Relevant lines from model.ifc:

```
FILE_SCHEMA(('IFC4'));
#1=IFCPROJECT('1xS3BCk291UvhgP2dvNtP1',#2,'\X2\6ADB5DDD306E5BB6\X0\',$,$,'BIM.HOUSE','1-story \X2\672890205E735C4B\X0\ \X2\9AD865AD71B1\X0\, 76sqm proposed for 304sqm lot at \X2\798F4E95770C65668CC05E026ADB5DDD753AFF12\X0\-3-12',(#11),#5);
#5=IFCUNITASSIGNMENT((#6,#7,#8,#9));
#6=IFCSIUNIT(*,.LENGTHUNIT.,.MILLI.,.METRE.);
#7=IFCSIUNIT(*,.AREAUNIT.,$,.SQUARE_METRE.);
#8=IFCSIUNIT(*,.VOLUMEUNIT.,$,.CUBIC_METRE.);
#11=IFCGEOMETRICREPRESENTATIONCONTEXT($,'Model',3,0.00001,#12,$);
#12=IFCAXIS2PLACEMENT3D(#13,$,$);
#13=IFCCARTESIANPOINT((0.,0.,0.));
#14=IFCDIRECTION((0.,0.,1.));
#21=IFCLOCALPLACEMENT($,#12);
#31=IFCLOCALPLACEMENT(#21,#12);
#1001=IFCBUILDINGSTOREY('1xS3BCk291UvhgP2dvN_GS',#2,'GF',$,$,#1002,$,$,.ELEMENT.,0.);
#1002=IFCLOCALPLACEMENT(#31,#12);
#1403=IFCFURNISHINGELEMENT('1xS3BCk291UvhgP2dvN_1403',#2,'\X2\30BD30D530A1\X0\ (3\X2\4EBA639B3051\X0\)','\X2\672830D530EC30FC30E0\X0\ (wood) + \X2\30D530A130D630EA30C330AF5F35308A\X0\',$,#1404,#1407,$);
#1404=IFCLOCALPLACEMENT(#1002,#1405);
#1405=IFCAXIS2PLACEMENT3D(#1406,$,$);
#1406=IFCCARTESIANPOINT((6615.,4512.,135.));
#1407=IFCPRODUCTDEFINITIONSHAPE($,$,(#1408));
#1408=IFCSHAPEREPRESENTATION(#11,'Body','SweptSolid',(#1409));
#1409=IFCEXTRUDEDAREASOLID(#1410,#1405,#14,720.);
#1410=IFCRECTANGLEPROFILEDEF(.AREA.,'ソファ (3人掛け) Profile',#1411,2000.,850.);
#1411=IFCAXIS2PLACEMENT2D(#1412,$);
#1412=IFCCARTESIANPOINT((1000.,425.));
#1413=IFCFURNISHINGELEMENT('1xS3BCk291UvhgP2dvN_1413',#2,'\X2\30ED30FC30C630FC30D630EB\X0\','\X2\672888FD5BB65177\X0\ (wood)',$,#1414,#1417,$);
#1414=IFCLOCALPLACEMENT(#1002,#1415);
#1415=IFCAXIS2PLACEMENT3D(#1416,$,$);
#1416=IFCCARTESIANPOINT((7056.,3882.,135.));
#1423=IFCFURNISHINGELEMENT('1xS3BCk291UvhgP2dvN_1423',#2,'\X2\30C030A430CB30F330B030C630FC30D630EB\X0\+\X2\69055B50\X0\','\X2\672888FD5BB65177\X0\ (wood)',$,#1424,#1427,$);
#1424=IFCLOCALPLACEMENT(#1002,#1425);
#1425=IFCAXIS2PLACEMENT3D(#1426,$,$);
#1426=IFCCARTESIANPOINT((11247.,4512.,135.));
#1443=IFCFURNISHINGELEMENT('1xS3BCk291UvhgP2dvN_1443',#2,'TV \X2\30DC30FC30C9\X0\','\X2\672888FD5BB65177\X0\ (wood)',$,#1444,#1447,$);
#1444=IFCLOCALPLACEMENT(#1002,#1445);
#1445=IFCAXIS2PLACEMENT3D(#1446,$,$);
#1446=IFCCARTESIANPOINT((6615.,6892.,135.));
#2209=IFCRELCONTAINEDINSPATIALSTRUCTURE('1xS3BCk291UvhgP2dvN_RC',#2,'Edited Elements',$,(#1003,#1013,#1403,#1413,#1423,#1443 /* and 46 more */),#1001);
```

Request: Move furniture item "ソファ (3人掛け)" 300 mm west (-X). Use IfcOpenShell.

```python
import ifcopenshell
import ifcopenshell.api.geometry
import ifcopenshell.util.placement
import ifcopenshell.util.unit

model = ifcopenshell.open("model.ifc")
unit_scale = ifcopenshell.util.unit.calculate_unit_scale(model)

item = model.by_id(1403)
matrix = ifcopenshell.util.placement.get_local_placement(item.ObjectPlacement)
matrix[0, 3] -= 0.3 / unit_scale
ifcopenshell.api.geometry.edit_object_placement(model, product=item, matrix=matrix, is_si=False)

print(ifcopenshell.util.placement.get_local_placement(item.ObjectPlacement).round(3) + 0.0)

model.write("model_rev.ifc")
```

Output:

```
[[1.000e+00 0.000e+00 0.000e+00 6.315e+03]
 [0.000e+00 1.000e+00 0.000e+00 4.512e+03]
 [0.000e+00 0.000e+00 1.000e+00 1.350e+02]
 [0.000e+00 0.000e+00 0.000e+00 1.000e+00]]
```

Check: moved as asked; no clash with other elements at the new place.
